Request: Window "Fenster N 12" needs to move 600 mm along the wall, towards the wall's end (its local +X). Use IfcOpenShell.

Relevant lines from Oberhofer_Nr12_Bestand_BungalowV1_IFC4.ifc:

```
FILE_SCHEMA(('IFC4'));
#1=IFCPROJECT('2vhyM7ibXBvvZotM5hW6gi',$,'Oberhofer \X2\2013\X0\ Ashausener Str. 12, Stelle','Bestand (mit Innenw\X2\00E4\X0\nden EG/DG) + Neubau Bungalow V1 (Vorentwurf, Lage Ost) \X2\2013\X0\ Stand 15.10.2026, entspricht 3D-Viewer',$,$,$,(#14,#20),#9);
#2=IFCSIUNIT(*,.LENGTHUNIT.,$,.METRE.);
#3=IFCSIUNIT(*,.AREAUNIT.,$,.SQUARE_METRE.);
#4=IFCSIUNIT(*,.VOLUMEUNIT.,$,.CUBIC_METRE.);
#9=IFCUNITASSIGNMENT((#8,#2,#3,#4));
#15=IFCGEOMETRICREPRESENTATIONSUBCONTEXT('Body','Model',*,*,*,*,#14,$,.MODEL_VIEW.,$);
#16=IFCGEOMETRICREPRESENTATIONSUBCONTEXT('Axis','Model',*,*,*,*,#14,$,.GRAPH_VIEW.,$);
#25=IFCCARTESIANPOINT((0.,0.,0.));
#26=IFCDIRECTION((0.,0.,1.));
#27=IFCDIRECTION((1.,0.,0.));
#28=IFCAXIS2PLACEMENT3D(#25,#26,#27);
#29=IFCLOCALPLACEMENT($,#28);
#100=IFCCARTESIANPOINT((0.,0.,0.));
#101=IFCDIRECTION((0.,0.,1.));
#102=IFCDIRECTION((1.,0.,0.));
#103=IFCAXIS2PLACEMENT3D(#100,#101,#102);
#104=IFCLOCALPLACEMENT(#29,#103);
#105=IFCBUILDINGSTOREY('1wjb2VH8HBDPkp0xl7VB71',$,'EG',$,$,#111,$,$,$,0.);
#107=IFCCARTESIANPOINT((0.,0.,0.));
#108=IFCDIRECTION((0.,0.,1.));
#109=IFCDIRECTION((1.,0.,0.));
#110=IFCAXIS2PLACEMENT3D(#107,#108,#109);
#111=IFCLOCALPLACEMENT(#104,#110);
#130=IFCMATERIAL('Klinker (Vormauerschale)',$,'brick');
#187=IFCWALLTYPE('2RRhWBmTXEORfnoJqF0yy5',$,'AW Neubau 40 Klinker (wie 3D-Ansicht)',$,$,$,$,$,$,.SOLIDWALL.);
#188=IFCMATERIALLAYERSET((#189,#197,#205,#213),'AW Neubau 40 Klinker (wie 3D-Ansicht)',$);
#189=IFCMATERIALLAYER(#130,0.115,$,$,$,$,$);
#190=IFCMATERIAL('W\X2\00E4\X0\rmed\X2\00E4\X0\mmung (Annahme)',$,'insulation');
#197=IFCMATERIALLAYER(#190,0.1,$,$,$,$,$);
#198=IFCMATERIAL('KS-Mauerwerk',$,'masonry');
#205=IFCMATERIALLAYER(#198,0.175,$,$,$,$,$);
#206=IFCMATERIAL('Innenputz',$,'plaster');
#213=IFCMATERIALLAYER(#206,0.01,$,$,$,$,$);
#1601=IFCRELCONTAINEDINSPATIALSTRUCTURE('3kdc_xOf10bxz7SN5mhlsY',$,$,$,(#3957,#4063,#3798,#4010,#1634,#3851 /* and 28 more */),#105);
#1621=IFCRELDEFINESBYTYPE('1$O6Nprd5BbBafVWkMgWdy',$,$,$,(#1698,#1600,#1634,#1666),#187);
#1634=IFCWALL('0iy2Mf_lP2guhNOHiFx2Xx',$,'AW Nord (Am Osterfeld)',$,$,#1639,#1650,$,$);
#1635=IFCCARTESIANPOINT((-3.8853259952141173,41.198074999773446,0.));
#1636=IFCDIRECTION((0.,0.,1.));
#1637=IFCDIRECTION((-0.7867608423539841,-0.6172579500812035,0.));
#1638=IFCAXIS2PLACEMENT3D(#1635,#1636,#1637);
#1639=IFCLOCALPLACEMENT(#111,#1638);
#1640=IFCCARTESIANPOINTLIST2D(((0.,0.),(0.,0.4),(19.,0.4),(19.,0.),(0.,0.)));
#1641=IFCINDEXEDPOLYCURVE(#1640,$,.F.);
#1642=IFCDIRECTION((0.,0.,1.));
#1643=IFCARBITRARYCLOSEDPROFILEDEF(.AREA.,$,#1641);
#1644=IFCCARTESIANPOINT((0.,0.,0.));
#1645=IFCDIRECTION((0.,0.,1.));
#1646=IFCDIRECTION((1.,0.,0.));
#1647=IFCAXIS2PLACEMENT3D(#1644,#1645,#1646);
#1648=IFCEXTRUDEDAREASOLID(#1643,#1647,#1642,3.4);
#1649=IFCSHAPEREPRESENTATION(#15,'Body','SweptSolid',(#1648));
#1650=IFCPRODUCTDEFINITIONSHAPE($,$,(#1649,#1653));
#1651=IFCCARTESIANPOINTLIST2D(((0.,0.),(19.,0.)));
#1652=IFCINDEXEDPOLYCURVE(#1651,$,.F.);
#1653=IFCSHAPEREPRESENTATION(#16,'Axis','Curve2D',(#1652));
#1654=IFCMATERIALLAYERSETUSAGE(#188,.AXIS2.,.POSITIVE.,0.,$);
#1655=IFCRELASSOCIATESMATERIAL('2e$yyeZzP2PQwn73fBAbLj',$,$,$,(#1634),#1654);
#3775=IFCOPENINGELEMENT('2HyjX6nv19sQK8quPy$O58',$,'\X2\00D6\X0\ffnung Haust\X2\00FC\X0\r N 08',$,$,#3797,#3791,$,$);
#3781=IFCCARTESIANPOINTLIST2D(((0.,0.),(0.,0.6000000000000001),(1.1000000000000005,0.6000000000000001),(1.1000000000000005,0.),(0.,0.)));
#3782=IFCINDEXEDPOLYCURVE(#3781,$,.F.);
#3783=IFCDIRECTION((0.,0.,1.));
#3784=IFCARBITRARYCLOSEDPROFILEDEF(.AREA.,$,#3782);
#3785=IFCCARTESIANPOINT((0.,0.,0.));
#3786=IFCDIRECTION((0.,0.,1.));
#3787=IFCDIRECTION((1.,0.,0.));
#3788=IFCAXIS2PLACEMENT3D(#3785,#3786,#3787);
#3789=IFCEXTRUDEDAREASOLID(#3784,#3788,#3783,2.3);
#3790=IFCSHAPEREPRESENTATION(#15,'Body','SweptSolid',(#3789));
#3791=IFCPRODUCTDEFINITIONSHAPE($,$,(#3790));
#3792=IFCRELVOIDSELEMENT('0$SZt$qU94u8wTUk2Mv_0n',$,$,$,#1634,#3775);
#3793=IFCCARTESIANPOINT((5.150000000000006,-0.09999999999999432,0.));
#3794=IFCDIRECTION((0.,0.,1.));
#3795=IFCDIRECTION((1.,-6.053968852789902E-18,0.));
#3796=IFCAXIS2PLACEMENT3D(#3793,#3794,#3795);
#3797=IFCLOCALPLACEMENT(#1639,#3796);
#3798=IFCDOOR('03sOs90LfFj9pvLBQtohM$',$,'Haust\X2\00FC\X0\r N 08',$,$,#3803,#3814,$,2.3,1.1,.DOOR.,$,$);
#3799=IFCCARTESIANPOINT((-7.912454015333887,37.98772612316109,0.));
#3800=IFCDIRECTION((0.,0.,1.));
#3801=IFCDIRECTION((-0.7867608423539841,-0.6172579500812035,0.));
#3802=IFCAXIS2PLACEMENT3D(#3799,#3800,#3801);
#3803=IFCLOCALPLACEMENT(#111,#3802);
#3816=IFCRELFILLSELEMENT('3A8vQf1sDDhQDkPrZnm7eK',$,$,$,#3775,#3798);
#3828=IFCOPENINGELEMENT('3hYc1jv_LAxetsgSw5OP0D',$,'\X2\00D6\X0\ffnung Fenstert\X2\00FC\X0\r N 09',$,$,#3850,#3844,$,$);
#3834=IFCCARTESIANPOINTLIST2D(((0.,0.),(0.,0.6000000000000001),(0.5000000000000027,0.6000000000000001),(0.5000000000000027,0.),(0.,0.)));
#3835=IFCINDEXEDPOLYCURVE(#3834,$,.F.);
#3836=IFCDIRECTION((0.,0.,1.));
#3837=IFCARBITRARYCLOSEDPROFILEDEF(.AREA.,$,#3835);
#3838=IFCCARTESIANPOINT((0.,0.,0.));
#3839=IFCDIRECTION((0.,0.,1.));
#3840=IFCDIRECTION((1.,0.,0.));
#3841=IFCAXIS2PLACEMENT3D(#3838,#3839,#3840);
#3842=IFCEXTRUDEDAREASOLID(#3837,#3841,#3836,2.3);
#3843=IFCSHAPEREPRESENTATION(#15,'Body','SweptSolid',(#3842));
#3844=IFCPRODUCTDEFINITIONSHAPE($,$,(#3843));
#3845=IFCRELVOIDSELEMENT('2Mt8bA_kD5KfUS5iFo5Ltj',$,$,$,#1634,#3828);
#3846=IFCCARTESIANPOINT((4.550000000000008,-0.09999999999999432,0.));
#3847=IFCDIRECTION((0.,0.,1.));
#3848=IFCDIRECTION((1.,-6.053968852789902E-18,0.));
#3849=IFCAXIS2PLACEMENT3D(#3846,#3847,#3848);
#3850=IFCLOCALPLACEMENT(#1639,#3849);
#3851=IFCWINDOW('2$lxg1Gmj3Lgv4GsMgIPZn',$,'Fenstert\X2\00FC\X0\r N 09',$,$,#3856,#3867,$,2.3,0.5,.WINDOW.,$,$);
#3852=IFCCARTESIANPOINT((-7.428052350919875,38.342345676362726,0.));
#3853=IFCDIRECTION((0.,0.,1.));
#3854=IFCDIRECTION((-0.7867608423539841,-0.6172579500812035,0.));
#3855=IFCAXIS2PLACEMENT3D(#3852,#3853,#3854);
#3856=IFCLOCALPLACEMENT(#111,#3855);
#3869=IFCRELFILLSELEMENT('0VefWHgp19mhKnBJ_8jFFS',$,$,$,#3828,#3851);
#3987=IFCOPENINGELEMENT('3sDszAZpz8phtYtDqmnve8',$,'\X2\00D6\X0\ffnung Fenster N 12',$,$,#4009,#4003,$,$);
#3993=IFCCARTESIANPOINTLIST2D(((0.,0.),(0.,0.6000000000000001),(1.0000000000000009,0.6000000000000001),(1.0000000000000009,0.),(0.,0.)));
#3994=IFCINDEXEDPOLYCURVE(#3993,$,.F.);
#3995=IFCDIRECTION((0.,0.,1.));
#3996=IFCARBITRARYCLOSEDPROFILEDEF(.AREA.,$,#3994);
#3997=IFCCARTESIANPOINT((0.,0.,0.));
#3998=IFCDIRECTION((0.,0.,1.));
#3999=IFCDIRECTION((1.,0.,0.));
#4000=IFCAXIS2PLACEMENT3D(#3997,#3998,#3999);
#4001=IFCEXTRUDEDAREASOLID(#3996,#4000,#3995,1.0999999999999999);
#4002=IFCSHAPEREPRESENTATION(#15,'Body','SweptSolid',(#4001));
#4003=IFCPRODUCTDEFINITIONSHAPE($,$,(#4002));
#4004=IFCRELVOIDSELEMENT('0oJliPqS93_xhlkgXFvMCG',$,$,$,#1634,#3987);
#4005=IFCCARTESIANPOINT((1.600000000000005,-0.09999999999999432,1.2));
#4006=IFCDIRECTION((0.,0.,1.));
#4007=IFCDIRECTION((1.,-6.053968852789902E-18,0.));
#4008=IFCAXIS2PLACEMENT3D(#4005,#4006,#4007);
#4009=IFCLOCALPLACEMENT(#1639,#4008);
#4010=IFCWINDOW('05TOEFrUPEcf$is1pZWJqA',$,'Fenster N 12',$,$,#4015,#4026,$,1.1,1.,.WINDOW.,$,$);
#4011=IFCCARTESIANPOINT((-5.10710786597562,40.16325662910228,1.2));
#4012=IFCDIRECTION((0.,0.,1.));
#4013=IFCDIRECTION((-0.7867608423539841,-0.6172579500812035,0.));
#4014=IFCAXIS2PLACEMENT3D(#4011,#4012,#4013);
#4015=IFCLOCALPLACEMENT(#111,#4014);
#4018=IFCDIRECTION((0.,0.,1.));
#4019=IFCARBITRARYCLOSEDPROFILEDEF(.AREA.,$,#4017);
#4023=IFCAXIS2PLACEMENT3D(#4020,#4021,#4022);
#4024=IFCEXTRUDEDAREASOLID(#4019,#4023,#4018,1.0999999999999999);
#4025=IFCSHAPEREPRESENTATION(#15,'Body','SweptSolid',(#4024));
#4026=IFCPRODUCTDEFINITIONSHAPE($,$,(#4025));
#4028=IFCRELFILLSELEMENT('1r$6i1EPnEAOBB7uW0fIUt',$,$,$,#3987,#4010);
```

```python
import ifcopenshell
import ifcopenshell.api.geometry
import ifcopenshell.util.placement
import ifcopenshell.util.unit

model = ifcopenshell.open("Oberhofer_Nr12_Bestand_BungalowV1_IFC4.ifc")
unit_scale = ifcopenshell.util.unit.calculate_unit_scale(model)

window = model.by_guid("05TOEFrUPEcf$is1pZWJqA")
opening = window.FillsVoids[0].RelatingOpeningElement
wall = opening.VoidsElements[0].RelatingBuildingElement

wall_matrix = ifcopenshell.util.placement.get_local_placement(wall.ObjectPlacement)
shift = wall_matrix[:3, 0] * 0.6 / unit_scale
before = ifcopenshell.util.placement.get_local_placement(window.ObjectPlacement)[:3, 3].copy()

# The window is not placed relative to its opening, so move both.
for product in (opening, window):
    matrix = ifcopenshell.util.placement.get_local_placement(product.ObjectPlacement)
    matrix[:3, 3] += shift
    ifcopenshell.api.geometry.edit_object_placement(model, product=product, matrix=matrix, is_si=False)

after = ifcopenshell.util.placement.get_local_placement(window.ObjectPlacement)[:3, 3]
print("window moved by", (after - before).round(3) + 0.0)

model.write("Oberhofer_Nr12_Bestand_BungalowV1_IFC4-out.ifc")
```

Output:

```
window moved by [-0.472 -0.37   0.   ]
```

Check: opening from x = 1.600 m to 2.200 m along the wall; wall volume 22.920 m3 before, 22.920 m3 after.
